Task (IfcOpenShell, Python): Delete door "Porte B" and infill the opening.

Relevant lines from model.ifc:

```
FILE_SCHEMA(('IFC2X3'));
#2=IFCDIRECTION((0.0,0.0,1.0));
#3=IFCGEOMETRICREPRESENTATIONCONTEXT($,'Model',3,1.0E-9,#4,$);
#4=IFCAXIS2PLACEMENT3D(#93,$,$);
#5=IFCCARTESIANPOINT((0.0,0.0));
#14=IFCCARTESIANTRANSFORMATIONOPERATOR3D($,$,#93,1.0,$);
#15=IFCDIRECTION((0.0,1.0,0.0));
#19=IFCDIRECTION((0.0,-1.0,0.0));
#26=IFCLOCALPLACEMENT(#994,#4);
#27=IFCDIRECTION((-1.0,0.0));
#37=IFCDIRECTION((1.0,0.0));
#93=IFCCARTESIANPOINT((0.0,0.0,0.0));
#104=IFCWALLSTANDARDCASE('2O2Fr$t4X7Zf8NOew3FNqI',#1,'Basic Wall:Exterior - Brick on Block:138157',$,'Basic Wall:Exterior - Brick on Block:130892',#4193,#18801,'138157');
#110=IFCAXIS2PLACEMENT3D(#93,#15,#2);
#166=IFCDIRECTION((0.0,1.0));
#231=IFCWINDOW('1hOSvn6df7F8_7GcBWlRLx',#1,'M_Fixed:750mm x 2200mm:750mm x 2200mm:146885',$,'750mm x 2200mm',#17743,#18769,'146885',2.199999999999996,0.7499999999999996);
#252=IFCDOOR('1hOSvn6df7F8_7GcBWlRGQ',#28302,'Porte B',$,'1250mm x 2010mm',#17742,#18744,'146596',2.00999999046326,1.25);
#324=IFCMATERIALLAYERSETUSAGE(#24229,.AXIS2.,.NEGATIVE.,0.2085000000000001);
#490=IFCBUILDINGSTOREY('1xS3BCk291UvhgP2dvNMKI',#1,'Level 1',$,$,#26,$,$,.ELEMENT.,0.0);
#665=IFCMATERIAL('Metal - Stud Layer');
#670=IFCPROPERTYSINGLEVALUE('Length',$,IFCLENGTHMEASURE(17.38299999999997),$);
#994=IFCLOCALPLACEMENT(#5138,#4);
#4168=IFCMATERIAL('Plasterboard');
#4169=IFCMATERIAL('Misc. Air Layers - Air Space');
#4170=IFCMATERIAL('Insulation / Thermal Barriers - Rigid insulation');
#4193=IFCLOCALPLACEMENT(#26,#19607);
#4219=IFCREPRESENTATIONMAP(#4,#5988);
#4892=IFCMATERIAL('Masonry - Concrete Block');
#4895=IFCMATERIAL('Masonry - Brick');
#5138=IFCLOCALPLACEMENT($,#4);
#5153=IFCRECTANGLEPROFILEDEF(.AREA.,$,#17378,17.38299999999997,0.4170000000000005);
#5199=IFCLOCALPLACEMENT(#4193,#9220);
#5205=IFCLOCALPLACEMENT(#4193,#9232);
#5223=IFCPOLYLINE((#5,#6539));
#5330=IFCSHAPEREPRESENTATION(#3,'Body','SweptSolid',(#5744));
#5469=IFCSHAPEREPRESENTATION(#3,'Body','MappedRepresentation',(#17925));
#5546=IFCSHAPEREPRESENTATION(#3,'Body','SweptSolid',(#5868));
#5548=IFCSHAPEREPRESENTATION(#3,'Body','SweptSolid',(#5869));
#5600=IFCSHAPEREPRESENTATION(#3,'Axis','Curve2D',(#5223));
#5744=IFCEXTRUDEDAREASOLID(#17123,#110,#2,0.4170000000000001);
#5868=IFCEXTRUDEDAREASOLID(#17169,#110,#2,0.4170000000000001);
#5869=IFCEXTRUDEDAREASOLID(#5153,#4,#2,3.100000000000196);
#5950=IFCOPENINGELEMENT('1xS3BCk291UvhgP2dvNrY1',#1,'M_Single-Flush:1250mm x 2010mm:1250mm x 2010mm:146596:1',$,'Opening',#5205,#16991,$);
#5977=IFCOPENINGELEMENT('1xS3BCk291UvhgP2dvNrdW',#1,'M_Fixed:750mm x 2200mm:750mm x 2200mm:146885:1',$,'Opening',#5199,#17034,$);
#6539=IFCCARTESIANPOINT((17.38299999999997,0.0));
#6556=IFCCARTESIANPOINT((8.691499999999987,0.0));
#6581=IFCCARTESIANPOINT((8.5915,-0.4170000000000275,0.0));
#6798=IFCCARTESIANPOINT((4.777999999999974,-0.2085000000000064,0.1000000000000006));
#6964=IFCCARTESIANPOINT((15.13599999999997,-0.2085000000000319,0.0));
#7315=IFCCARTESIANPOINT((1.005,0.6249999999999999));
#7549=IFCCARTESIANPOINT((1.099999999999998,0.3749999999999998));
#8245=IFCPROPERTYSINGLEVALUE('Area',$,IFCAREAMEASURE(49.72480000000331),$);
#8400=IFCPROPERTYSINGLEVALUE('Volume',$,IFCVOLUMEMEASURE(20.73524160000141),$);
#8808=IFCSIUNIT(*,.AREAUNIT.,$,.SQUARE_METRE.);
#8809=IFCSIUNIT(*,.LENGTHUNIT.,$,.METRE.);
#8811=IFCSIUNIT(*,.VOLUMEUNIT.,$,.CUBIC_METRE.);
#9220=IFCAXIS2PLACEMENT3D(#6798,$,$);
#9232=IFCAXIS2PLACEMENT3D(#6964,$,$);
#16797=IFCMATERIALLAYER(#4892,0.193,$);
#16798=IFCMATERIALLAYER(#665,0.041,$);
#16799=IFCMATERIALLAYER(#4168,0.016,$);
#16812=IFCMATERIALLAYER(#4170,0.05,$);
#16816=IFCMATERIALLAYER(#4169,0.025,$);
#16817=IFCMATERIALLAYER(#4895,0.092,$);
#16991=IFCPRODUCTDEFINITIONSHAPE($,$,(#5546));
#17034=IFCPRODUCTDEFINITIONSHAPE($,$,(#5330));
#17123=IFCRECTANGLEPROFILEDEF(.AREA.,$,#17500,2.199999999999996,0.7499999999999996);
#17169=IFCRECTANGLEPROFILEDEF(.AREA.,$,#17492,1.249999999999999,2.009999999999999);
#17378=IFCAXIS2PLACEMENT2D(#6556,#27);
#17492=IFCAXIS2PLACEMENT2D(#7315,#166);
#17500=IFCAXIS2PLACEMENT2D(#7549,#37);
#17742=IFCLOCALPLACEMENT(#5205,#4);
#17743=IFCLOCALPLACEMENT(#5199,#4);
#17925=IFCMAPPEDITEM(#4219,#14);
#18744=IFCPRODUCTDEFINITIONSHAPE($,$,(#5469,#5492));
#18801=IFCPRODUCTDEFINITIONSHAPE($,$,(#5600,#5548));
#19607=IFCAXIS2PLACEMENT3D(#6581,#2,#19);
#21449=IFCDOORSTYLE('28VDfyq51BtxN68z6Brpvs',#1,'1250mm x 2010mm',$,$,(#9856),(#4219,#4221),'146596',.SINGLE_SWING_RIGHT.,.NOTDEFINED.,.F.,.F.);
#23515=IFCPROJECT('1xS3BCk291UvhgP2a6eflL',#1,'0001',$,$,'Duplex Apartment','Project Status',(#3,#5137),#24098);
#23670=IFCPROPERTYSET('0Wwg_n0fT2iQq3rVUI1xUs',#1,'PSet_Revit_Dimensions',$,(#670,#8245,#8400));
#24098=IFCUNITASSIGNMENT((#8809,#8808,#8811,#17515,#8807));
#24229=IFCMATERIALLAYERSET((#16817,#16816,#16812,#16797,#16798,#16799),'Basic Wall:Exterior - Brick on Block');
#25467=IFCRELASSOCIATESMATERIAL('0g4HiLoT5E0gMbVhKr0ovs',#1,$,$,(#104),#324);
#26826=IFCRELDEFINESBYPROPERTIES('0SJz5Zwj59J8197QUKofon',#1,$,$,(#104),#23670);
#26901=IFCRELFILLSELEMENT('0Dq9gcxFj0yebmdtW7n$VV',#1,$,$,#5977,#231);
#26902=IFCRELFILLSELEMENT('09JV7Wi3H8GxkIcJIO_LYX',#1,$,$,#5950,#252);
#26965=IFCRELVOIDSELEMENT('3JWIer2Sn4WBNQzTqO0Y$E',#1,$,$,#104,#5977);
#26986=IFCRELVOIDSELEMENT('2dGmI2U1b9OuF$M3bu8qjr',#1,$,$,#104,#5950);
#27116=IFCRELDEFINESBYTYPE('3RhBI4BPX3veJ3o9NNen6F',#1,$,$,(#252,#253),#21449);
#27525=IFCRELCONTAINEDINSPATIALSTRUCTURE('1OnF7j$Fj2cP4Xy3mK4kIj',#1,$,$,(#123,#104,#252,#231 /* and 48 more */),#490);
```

```python
import ifcopenshell
import ifcopenshell.api.feature
import ifcopenshell.api.pset
import ifcopenshell.api.root
import ifcopenshell.geom
import ifcopenshell.util.element
import ifcopenshell.util.shape
import ifcopenshell.util.unit

model = ifcopenshell.open("model.ifc")
area_scale = ifcopenshell.util.unit.calculate_unit_scale(model, "AREAUNIT")
volume_scale = ifcopenshell.util.unit.calculate_unit_scale(model, "VOLUMEUNIT")
settings = ifcopenshell.geom.settings()


def volume(element):
    """Net volume in cubic metres, openings subtracted."""
    shape = ifcopenshell.geom.create_shape(settings, element)
    return ifcopenshell.util.shape.get_volume(shape.geometry)


door = model.by_guid("1hOSvn6df7F8_7GcBWlRGQ")
opening = door.FillsVoids[0].RelatingOpeningElement
wall = opening.VoidsElements[0].RelatingBuildingElement
before = volume(wall)

ifcopenshell.api.root.remove_product(model, product=door)
ifcopenshell.api.feature.remove_feature(model, feature=opening)

after = volume(wall)
thickness = 0.417  # wall thickness in metres

# Update the wall's stored quantities.
pset = model.by_id(ifcopenshell.util.element.get_pset(wall, "PSet_Revit_Dimensions", should_inherit=False)["id"])
ifcopenshell.api.pset.edit_pset(model, pset=pset, properties={
    "Area": model.create_entity("IfcAreaMeasure", after / thickness / area_scale),
    "Volume": model.create_entity("IfcVolumeMeasure", after / volume_scale),
})

print(f"wall volume {before:.3f} -> {after:.3f} m3")

model.write("model_v2.ifc")
```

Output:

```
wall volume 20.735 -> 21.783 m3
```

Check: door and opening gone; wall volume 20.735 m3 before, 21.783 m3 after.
